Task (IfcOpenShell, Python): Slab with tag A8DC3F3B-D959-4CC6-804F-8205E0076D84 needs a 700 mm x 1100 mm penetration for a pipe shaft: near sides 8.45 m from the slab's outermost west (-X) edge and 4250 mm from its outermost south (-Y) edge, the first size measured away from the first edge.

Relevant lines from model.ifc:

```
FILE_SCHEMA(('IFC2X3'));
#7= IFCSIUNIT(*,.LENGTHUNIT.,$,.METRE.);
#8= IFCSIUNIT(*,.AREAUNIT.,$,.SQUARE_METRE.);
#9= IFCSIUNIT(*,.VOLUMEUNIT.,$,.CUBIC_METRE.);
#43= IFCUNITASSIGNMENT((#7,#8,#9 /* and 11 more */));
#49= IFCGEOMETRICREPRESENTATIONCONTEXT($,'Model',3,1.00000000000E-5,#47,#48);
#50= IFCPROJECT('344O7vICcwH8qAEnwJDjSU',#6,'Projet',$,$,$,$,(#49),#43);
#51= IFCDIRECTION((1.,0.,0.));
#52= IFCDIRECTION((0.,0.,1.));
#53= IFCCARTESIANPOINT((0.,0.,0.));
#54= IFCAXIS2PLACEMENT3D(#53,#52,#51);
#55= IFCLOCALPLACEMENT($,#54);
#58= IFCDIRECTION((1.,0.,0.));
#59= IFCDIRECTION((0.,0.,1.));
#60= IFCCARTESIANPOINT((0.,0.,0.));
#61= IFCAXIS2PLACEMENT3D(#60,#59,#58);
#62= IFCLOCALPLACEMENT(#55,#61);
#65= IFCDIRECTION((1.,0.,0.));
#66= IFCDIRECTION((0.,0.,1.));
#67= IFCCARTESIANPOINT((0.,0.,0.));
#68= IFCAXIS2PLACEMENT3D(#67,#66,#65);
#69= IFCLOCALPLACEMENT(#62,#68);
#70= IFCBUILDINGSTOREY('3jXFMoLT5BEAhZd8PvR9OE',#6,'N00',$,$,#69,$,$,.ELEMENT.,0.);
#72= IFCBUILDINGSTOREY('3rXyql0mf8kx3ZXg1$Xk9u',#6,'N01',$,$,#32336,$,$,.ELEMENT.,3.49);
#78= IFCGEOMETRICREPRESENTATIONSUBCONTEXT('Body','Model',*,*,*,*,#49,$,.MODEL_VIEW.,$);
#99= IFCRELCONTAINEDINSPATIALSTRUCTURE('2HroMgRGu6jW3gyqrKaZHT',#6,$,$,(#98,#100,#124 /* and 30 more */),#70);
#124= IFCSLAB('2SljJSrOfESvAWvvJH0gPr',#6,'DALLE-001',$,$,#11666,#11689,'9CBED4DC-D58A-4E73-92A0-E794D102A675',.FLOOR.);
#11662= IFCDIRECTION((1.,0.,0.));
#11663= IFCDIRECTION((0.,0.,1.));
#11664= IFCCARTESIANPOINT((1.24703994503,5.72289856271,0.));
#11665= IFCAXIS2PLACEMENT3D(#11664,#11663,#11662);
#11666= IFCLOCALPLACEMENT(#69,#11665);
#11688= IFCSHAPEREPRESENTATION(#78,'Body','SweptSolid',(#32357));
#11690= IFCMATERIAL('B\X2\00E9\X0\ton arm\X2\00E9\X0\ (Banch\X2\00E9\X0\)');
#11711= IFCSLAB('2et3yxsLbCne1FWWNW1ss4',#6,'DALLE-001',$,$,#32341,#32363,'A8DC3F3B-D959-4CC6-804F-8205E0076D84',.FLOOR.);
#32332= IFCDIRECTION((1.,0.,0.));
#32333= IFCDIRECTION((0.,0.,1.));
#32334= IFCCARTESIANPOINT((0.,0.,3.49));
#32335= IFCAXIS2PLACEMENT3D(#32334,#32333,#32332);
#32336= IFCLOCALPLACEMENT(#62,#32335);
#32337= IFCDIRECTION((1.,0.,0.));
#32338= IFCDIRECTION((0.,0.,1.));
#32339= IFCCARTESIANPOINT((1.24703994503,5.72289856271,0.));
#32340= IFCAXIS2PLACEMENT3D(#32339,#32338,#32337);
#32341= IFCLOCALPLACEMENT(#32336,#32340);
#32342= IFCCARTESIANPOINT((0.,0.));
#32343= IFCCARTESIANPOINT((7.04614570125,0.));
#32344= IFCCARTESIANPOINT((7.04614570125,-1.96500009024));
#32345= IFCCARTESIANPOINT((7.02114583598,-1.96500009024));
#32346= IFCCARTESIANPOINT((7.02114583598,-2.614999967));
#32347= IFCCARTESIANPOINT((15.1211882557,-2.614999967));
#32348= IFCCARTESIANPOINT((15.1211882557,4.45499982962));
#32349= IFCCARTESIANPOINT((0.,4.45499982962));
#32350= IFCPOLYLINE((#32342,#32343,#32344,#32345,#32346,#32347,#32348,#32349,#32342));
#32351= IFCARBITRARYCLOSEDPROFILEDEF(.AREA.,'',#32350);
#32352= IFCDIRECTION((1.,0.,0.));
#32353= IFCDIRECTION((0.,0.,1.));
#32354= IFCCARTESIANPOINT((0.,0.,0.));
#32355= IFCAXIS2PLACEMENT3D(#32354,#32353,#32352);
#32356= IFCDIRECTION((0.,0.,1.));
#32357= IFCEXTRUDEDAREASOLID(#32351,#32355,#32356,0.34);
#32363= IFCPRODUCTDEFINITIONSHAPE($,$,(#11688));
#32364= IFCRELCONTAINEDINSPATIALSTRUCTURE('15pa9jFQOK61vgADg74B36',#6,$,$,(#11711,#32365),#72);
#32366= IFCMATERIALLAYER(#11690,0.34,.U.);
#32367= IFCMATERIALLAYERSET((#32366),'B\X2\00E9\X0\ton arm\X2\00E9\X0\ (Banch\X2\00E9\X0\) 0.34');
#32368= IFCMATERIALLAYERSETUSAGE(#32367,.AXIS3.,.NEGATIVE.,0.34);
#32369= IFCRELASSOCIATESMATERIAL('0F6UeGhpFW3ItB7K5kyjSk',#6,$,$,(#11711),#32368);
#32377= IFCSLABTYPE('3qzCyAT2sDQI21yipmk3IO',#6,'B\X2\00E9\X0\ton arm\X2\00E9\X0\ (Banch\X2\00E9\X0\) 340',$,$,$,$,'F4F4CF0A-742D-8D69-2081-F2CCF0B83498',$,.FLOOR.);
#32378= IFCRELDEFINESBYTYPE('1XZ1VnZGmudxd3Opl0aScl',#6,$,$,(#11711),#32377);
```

```python
import numpy as np
import ifcopenshell
import ifcopenshell.api.feature
import ifcopenshell.api.geometry
import ifcopenshell.api.root
import ifcopenshell.geom
import ifcopenshell.util.placement
import ifcopenshell.util.representation
import ifcopenshell.util.shape
import ifcopenshell.util.unit

model = ifcopenshell.open("model.ifc")
unit_scale = ifcopenshell.util.unit.calculate_unit_scale(model)
settings = ifcopenshell.geom.settings()


def volume(element):
    """Net volume in cubic metres, openings subtracted."""
    shape = ifcopenshell.geom.create_shape(settings, element)
    return ifcopenshell.util.shape.get_volume(shape.geometry)


slab = model.by_guid("2et3yxsLbCne1FWWNW1ss4")
before = volume(slab)

# Extent in the slab's own axes, in metres. The edges named are its -X and -Y sides.
slab_shape = ifcopenshell.geom.create_shape(settings, slab)
vertices = ifcopenshell.util.shape.get_vertices(slab_shape.geometry)
x_min, y_min, bottom = vertices.min(axis=0)
top = vertices[:, 2].max()

opening = ifcopenshell.api.root.create_entity(model, ifc_class="IfcOpeningElement", name="Pipe shaft opening")
context = ifcopenshell.util.representation.get_context(model, "Model", "Body", "MODEL_VIEW")
width, depth = 0.7, 1.1
outline = [(0.0, 0.0), (width, 0.0), (width, depth), (0.0, depth), (0.0, 0.0)]
# Overshoot both faces by 50 mm so the cut is clean.
shape = ifcopenshell.api.geometry.add_slab_representation(
    model, context=context, depth=top - bottom + 0.1, polyline=outline
)
ifcopenshell.api.geometry.assign_representation(model, product=opening, representation=shape)

matrix = ifcopenshell.util.placement.get_local_placement(slab.ObjectPlacement)
matrix[:, 3] = matrix @ np.append(np.array([x_min + 8.45, y_min + 4.25, bottom - 0.05]) / unit_scale, 1.0)
ifcopenshell.api.geometry.edit_object_placement(model, product=opening, matrix=matrix, is_si=False)
ifcopenshell.api.feature.add_feature(model, feature=opening, element=slab)

after = volume(slab)

print(f"slab volume {before:.3f} -> {after:.3f} m3")

model.write("model_rev.ifc")
```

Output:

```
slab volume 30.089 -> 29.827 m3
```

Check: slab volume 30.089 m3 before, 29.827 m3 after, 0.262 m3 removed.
